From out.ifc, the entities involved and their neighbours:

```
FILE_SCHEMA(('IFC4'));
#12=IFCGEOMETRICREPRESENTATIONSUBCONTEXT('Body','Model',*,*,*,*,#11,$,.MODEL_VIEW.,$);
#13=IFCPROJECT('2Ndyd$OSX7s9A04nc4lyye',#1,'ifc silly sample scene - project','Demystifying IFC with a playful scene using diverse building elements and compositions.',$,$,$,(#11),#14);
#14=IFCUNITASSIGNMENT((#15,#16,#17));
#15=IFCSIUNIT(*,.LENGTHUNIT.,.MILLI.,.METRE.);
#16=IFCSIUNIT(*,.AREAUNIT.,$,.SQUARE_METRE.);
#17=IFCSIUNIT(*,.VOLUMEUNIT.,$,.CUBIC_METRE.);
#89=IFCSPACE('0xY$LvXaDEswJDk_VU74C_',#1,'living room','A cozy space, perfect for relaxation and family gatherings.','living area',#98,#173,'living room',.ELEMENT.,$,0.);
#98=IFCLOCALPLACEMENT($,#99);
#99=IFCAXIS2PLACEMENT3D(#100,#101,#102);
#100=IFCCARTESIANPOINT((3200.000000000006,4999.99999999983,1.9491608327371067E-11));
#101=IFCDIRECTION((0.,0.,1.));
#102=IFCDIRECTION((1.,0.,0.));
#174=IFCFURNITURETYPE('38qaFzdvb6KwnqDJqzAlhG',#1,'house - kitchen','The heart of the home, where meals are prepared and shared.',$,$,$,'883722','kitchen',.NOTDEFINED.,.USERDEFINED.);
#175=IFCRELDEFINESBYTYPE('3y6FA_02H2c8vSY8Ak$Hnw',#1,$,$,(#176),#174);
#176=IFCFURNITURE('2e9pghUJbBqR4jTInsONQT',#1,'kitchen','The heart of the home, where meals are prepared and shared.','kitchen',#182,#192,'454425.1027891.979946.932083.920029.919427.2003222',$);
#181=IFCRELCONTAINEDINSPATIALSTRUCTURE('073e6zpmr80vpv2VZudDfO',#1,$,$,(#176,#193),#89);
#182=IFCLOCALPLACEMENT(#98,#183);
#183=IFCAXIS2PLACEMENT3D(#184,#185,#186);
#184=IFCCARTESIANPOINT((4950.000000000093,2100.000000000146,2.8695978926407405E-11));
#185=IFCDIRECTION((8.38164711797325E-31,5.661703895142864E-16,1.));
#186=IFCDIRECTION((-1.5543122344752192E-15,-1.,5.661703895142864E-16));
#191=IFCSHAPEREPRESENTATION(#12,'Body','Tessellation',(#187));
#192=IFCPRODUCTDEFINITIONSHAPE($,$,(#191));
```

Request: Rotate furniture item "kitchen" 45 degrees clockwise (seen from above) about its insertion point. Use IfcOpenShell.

```python
import ifcopenshell
import ifcopenshell.api.geometry
import ifcopenshell.util.placement

model = ifcopenshell.open("out.ifc")

item = model.by_guid("2e9pghUJbBqR4jTInsONQT")
matrix = ifcopenshell.util.placement.get_local_placement(item.ObjectPlacement)
matrix = matrix @ ifcopenshell.util.placement.rotation(-45, "Z")
ifcopenshell.api.geometry.edit_object_placement(model, product=item, matrix=matrix, is_si=False)

print(ifcopenshell.util.placement.get_local_placement(item.ObjectPlacement).round(3) + 0.0)

model.write("out-out.ifc")
```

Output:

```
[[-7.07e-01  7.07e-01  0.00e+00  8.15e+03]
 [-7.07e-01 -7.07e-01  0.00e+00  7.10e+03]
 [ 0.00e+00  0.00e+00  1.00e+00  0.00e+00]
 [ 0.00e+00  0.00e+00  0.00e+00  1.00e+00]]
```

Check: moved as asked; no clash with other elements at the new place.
